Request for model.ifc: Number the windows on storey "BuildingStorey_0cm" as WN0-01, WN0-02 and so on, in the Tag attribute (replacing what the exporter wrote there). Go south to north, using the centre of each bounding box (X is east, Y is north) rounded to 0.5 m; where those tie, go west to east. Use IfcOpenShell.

First a look at what the model holds.

```python
import ifcopenshell
import ifcopenshell.util.element
import ifcopenshell.util.placement

model = ifcopenshell.open("model.ifc")
print(model.schema)
storey = next(s for s in model.by_type("IfcBuildingStorey") if s.Name == "BuildingStorey_0cm")
windows = [e for e in ifcopenshell.util.element.get_decomposition(storey) if e.is_a("IfcWindow")]
for e in sorted(windows, key=lambda e: e.id()):
    origin = ifcopenshell.util.placement.get_local_placement(e.ObjectPlacement)[:3, 3]
    print(e.id(), e.Tag, e.Name, origin.round(2) + 0.0, sep=" | ")
```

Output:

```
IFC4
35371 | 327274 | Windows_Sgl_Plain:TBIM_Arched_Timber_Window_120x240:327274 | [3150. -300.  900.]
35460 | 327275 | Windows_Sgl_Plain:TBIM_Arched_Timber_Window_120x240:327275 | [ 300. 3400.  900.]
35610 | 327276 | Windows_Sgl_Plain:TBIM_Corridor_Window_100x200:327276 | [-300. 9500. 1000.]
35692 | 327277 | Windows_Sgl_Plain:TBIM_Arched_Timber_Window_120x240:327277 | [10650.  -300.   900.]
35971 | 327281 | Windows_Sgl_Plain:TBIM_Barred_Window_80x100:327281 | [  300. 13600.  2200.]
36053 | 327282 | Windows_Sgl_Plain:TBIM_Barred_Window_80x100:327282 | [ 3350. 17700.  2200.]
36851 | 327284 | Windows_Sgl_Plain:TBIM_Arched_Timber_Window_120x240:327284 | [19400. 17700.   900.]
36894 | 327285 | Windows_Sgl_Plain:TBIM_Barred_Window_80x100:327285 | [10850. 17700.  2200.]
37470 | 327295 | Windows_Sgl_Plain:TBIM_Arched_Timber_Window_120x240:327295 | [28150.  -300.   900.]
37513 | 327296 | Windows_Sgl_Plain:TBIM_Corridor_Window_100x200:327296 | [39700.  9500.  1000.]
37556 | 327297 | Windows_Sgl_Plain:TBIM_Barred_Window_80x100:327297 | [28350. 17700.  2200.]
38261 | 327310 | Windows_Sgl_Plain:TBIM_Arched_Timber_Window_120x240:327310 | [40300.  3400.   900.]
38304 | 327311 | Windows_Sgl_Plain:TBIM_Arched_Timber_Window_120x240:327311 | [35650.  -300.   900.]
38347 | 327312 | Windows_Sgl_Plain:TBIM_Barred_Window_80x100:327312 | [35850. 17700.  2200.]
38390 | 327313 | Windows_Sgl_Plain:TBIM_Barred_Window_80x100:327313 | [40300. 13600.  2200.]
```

```python
import ifcopenshell
import ifcopenshell.geom
import ifcopenshell.util.element
import ifcopenshell.util.shape

model = ifcopenshell.open("model.ifc")
settings = ifcopenshell.geom.settings()
settings.set("use-world-coords", True)


def centre(element):
    shape = ifcopenshell.geom.create_shape(settings, element)
    return ifcopenshell.util.shape.get_bbox_centroid(shape.geometry)


storey = next(s for s in model.by_type("IfcBuildingStorey") if s.Name == "BuildingStorey_0cm")
windows = [e for e in ifcopenshell.util.element.get_decomposition(storey) if e.is_a("IfcWindow")]

# Insertion points can sit at a corner or the storey origin, so sort by the geometry (in metres).
centres = {e: centre(e) for e in windows}
windows.sort(key=lambda e: (round(centres[e][1] / 0.5), centres[e][0]))

for i, e in enumerate(windows, start=1):
    number = f"WN0-{i:02d}"
    e.Tag = number
    print(e.id(), number)

model.write("model-out.ifc")
```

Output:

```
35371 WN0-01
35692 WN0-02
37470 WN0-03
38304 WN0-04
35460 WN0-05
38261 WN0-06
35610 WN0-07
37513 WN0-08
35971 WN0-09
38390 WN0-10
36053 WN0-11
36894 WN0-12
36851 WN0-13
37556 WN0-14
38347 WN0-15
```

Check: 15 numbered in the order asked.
